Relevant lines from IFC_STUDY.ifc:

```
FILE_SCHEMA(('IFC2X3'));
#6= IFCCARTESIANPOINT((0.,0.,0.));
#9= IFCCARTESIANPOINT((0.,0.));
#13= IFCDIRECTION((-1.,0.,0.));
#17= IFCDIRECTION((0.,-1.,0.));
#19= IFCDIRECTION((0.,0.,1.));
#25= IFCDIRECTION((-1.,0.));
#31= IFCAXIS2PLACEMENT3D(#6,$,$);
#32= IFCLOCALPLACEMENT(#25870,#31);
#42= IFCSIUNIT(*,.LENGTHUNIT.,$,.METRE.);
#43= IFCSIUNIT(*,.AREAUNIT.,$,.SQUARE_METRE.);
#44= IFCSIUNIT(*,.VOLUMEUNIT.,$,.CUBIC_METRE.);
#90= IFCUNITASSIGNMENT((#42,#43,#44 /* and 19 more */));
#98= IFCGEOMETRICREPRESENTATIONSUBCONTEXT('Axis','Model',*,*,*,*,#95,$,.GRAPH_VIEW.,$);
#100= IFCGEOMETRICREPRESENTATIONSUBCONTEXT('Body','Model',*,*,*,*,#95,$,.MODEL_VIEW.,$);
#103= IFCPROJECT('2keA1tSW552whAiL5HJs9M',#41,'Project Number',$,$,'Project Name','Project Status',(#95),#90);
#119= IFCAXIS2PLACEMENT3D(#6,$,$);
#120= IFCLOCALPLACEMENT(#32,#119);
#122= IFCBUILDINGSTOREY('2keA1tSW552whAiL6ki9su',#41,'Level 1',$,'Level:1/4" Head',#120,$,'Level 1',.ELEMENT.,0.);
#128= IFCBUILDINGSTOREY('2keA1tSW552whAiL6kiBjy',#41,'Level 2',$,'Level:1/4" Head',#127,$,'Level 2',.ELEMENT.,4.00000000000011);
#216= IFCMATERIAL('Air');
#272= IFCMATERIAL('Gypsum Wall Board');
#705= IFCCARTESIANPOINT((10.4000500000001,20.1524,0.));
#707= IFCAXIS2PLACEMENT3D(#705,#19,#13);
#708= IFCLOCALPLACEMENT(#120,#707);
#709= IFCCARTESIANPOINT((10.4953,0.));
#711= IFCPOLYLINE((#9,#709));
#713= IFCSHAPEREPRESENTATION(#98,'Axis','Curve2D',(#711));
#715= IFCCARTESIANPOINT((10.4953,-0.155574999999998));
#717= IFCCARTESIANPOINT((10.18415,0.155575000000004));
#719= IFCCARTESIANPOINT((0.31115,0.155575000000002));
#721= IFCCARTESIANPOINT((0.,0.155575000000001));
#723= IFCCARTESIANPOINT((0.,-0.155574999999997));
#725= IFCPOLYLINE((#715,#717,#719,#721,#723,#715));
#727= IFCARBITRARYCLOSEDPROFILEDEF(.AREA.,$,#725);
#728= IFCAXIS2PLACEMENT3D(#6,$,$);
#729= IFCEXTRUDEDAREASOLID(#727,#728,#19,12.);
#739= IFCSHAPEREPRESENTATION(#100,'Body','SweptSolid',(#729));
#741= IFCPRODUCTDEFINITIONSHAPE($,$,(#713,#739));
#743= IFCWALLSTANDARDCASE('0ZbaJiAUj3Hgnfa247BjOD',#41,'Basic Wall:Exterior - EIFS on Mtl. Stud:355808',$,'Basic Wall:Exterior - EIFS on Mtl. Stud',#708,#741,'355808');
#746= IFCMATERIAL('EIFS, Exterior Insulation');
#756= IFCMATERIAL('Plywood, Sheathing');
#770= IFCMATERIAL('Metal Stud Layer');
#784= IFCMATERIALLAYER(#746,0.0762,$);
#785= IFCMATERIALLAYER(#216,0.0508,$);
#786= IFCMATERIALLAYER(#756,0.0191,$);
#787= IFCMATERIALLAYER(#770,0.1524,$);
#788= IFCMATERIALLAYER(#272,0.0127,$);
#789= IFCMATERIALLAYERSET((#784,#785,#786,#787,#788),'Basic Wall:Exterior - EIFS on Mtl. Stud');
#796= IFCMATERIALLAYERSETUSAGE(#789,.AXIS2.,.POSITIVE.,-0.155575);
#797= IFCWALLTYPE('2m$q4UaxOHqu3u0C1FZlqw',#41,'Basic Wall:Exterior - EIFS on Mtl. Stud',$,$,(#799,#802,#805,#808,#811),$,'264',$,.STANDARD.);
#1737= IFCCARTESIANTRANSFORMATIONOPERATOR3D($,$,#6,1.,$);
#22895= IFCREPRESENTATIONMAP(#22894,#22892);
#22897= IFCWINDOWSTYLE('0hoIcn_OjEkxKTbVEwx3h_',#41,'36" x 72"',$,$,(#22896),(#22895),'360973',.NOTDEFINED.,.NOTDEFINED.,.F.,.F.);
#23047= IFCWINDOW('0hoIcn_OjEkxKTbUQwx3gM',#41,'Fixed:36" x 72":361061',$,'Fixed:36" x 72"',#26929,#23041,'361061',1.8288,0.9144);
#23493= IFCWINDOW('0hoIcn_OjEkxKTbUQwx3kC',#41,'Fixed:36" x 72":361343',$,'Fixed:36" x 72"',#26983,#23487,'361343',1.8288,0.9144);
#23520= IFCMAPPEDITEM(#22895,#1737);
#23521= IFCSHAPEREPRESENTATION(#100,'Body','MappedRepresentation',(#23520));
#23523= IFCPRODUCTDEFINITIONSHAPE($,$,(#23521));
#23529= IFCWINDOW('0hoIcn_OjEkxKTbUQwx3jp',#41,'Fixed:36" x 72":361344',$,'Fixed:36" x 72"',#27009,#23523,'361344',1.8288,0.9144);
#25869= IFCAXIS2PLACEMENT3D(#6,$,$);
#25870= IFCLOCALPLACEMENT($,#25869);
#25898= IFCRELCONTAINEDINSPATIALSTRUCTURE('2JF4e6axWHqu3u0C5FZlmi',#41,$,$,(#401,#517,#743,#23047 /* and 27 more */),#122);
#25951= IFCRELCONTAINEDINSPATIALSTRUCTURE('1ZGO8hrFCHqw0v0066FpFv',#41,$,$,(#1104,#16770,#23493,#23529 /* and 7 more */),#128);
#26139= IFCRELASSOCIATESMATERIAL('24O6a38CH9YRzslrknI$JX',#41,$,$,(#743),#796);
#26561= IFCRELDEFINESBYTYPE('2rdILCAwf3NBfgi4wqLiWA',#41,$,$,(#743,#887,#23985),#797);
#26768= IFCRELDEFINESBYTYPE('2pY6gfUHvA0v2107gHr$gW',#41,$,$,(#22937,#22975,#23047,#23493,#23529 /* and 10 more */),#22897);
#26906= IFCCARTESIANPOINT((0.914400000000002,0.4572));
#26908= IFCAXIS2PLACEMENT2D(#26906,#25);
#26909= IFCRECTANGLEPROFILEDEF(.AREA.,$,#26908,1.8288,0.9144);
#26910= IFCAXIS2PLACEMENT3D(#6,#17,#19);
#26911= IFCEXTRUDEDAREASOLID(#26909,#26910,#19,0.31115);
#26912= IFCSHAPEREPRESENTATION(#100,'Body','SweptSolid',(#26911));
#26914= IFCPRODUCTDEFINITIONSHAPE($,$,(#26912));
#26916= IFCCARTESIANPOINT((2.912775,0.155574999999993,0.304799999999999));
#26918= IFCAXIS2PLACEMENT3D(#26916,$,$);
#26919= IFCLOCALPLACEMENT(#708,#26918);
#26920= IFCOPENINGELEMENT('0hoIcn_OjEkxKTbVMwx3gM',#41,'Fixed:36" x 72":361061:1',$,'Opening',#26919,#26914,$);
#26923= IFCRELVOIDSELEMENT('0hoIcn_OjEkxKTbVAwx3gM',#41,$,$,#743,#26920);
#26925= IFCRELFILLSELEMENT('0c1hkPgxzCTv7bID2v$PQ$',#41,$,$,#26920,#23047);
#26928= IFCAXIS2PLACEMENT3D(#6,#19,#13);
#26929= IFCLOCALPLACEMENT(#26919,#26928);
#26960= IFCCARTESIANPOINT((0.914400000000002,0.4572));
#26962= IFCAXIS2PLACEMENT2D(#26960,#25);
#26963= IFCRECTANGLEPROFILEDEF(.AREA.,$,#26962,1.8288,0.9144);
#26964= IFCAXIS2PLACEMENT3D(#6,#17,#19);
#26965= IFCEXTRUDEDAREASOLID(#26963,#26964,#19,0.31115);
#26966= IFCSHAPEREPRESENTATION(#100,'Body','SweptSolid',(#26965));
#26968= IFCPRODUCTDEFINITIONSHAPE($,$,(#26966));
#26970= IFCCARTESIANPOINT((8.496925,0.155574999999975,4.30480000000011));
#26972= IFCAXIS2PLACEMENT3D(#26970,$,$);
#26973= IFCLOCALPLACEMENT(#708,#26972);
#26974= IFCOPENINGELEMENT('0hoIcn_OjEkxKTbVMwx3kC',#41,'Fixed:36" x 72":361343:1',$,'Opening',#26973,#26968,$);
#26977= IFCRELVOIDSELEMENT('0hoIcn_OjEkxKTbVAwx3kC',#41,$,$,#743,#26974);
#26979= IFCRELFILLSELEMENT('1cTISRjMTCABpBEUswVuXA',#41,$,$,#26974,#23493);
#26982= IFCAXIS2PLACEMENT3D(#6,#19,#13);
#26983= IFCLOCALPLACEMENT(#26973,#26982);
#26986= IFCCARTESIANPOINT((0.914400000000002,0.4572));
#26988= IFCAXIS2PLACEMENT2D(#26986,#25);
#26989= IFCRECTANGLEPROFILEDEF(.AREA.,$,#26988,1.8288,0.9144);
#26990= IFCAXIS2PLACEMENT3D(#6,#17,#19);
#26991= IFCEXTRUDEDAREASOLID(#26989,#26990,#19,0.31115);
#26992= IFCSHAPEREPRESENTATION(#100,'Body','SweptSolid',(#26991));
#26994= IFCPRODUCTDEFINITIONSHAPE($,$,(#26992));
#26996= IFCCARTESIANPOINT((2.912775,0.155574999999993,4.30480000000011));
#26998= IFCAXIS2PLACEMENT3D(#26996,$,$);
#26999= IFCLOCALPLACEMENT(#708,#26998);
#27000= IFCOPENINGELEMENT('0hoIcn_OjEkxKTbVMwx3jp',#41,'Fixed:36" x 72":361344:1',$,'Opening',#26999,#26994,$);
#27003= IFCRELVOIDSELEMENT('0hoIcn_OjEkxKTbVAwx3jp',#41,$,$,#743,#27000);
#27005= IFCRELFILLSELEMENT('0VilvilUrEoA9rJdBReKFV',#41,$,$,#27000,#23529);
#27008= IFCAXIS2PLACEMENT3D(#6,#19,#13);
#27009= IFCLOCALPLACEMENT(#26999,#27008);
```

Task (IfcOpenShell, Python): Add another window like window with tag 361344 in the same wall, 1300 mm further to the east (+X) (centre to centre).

```python
import ifcopenshell
import ifcopenshell.api.feature
import ifcopenshell.api.geometry
import ifcopenshell.api.root
import ifcopenshell.geom
import ifcopenshell.util.element
import ifcopenshell.util.placement
import ifcopenshell.util.shape
import ifcopenshell.util.unit

model = ifcopenshell.open("IFC_STUDY.ifc")
unit_scale = ifcopenshell.util.unit.calculate_unit_scale(model)
settings = ifcopenshell.geom.settings()


def volume(element):
    """Net volume in cubic metres, openings subtracted."""
    shape = ifcopenshell.geom.create_shape(settings, element)
    return ifcopenshell.util.shape.get_volume(shape.geometry)


def reuse_history(source, copy):
    """copy_class also copies each property set's owner history, people and application; keep the originals."""
    for rel in copy.IsDefinedBy:
        if rel.is_a("IfcRelDefinesByProperties") and (history := rel.RelatingPropertyDefinition.OwnerHistory):
            rel.RelatingPropertyDefinition.OwnerHistory = source.OwnerHistory
            ifcopenshell.util.element.remove_deep2(model, history)


window = model.by_guid("0hoIcn_OjEkxKTbUQwx3jp")
opening = window.FillsVoids[0].RelatingOpeningElement
wall = opening.VoidsElements[0].RelatingBuildingElement
before = volume(wall)
shift = ifcopenshell.util.placement.get_local_placement(wall.ObjectPlacement)[:3, 0] * -1.3 / unit_scale

# copy_class copies the void relationship, type, container and properties, but no geometry.
new_opening = ifcopenshell.api.root.copy_class(model, product=opening)
new_opening.Representation = ifcopenshell.util.element.copy_deep(
    model, opening.Representation, exclude=["IfcGeometricRepresentationContext", "IfcRepresentationMap"]
)
new_opening.Name = 'Fixed:36" x 72"'
new_window = ifcopenshell.api.root.copy_class(model, product=window)
new_window.Representation = ifcopenshell.util.element.copy_deep(
    model, window.Representation, exclude=["IfcGeometricRepresentationContext", "IfcRepresentationMap"]
)
new_window.Name = 'Fixed:36" x 72"'
new_window.Tag = None
reuse_history(window, new_window)
fills = ifcopenshell.api.feature.add_filling(model, opening=new_opening, element=new_window)
fills.OwnerHistory = new_window.OwnerHistory  # required in IFC2X3

for old, new in ((opening, new_opening), (window, new_window)):
    matrix = ifcopenshell.util.placement.get_local_placement(old.ObjectPlacement)
    matrix[:3, 3] += shift
    ifcopenshell.api.geometry.edit_object_placement(model, product=new, matrix=matrix, is_si=False)

after = volume(wall)

print(f"wall volume {before:.3f} -> {after:.3f} m3")

model.write("IFC_STUDY_rev.ifc")
```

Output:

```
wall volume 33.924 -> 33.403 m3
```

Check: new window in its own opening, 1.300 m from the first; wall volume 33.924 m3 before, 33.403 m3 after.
